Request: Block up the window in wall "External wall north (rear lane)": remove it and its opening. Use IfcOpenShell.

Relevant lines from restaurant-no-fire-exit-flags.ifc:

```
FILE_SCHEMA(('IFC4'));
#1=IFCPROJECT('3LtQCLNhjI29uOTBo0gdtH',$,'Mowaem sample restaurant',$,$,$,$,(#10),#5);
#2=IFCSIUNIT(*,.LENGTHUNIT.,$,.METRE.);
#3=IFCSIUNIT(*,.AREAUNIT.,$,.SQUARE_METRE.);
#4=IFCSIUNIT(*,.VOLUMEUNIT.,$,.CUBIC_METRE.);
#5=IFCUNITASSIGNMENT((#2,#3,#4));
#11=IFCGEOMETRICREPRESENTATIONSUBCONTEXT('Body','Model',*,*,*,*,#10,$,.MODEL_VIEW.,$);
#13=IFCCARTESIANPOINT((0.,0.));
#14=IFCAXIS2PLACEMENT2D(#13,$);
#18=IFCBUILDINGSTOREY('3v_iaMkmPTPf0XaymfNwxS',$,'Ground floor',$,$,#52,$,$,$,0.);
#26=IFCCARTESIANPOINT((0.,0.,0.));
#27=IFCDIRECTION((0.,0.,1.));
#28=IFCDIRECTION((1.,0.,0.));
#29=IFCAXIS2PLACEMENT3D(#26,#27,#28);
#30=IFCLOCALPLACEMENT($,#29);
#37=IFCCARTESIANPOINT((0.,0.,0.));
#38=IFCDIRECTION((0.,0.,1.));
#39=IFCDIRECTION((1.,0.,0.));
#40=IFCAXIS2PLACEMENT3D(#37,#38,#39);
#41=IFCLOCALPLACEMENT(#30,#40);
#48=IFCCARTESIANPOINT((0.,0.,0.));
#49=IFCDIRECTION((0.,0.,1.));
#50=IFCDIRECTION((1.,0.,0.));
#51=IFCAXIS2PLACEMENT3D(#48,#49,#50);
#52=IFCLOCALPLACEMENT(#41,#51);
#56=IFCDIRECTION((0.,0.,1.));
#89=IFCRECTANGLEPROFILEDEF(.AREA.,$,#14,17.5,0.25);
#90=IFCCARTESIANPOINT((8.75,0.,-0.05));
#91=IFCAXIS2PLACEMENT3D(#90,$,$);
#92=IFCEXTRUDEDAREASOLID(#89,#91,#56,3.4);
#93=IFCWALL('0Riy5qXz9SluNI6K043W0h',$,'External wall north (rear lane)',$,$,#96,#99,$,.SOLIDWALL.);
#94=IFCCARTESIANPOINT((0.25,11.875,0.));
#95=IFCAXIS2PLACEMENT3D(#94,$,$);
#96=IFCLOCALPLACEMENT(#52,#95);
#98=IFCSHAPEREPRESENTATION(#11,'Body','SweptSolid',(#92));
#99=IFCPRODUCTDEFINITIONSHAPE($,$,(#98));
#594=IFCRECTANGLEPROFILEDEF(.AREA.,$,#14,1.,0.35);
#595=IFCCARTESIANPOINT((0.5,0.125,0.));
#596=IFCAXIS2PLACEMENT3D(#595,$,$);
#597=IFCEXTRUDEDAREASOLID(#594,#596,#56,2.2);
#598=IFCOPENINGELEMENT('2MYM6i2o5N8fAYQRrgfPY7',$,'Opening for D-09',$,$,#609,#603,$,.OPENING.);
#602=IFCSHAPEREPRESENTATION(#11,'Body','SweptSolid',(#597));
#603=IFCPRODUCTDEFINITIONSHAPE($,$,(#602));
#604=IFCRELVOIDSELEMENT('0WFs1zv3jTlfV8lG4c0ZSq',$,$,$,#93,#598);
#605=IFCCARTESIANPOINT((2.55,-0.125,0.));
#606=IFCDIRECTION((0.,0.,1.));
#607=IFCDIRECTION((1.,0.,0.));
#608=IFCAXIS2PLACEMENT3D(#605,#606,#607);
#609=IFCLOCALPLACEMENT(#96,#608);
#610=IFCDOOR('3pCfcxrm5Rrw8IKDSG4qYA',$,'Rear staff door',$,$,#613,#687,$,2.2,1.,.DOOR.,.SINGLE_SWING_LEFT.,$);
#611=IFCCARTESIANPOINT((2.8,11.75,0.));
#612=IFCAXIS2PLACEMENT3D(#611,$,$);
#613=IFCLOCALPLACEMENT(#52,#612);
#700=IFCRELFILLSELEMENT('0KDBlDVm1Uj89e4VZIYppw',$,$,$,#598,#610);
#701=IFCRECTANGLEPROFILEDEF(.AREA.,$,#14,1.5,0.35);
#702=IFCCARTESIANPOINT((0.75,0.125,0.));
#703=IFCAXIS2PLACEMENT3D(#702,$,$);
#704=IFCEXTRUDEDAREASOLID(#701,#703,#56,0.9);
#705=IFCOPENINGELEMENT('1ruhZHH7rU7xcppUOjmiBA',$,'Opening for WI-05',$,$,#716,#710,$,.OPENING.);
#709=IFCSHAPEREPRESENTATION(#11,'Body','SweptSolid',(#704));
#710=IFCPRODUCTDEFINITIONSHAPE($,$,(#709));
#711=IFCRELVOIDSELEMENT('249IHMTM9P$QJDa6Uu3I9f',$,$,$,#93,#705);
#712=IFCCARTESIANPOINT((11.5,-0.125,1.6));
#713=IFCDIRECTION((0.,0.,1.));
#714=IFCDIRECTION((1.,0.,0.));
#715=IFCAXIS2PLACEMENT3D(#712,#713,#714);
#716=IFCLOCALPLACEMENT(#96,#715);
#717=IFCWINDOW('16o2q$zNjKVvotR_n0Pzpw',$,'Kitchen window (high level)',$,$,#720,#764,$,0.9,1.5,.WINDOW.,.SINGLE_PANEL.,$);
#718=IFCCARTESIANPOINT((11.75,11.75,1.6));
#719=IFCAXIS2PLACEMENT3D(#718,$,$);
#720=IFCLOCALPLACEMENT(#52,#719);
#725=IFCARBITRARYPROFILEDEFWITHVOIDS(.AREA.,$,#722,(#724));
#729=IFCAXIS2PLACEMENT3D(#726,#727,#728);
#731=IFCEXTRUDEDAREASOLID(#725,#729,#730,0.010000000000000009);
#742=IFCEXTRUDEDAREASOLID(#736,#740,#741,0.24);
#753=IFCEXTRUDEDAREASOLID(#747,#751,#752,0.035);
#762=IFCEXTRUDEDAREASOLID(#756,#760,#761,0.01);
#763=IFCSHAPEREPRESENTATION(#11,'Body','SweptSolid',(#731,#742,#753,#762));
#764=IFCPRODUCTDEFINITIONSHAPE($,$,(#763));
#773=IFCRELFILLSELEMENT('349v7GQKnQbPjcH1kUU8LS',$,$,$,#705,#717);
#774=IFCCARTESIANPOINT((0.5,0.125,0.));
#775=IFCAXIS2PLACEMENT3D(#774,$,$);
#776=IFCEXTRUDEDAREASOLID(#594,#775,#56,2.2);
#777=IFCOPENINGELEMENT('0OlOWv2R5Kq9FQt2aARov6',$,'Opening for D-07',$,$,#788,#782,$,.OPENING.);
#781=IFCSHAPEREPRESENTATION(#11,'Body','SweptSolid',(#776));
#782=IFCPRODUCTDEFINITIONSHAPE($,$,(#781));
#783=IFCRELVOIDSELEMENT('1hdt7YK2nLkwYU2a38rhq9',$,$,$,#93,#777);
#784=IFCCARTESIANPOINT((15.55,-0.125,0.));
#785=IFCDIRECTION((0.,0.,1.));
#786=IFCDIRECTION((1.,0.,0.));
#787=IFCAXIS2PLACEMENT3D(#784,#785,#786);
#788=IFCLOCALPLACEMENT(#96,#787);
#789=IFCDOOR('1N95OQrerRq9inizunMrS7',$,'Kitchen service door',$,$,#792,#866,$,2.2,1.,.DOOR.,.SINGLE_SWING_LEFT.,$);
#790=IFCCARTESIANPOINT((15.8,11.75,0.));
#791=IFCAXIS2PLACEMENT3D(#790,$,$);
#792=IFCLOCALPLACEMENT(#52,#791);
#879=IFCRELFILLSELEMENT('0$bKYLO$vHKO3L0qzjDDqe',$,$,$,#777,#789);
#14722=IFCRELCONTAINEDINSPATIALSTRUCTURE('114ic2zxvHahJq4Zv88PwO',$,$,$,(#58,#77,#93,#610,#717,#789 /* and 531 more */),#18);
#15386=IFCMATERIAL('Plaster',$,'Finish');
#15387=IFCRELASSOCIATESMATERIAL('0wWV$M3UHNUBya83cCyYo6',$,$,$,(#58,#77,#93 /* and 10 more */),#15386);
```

```python
import ifcopenshell
import ifcopenshell.api.feature
import ifcopenshell.api.root
import ifcopenshell.geom
import ifcopenshell.util.shape

model = ifcopenshell.open("restaurant-no-fire-exit-flags.ifc")
settings = ifcopenshell.geom.settings()


def volume(element):
    """Net volume in cubic metres, openings subtracted."""
    shape = ifcopenshell.geom.create_shape(settings, element)
    return ifcopenshell.util.shape.get_volume(shape.geometry)


window = model.by_id(717)
opening = window.FillsVoids[0].RelatingOpeningElement
wall = opening.VoidsElements[0].RelatingBuildingElement
before = volume(wall)

ifcopenshell.api.root.remove_product(model, product=window)
ifcopenshell.api.feature.remove_feature(model, feature=opening)

after = volume(wall)

print(f"wall volume {before:.3f} -> {after:.3f} m3")

model.write("restaurant-no-fire-exit-flags_updated.ifc")
```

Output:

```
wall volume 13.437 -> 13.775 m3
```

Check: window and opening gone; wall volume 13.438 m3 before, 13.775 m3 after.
